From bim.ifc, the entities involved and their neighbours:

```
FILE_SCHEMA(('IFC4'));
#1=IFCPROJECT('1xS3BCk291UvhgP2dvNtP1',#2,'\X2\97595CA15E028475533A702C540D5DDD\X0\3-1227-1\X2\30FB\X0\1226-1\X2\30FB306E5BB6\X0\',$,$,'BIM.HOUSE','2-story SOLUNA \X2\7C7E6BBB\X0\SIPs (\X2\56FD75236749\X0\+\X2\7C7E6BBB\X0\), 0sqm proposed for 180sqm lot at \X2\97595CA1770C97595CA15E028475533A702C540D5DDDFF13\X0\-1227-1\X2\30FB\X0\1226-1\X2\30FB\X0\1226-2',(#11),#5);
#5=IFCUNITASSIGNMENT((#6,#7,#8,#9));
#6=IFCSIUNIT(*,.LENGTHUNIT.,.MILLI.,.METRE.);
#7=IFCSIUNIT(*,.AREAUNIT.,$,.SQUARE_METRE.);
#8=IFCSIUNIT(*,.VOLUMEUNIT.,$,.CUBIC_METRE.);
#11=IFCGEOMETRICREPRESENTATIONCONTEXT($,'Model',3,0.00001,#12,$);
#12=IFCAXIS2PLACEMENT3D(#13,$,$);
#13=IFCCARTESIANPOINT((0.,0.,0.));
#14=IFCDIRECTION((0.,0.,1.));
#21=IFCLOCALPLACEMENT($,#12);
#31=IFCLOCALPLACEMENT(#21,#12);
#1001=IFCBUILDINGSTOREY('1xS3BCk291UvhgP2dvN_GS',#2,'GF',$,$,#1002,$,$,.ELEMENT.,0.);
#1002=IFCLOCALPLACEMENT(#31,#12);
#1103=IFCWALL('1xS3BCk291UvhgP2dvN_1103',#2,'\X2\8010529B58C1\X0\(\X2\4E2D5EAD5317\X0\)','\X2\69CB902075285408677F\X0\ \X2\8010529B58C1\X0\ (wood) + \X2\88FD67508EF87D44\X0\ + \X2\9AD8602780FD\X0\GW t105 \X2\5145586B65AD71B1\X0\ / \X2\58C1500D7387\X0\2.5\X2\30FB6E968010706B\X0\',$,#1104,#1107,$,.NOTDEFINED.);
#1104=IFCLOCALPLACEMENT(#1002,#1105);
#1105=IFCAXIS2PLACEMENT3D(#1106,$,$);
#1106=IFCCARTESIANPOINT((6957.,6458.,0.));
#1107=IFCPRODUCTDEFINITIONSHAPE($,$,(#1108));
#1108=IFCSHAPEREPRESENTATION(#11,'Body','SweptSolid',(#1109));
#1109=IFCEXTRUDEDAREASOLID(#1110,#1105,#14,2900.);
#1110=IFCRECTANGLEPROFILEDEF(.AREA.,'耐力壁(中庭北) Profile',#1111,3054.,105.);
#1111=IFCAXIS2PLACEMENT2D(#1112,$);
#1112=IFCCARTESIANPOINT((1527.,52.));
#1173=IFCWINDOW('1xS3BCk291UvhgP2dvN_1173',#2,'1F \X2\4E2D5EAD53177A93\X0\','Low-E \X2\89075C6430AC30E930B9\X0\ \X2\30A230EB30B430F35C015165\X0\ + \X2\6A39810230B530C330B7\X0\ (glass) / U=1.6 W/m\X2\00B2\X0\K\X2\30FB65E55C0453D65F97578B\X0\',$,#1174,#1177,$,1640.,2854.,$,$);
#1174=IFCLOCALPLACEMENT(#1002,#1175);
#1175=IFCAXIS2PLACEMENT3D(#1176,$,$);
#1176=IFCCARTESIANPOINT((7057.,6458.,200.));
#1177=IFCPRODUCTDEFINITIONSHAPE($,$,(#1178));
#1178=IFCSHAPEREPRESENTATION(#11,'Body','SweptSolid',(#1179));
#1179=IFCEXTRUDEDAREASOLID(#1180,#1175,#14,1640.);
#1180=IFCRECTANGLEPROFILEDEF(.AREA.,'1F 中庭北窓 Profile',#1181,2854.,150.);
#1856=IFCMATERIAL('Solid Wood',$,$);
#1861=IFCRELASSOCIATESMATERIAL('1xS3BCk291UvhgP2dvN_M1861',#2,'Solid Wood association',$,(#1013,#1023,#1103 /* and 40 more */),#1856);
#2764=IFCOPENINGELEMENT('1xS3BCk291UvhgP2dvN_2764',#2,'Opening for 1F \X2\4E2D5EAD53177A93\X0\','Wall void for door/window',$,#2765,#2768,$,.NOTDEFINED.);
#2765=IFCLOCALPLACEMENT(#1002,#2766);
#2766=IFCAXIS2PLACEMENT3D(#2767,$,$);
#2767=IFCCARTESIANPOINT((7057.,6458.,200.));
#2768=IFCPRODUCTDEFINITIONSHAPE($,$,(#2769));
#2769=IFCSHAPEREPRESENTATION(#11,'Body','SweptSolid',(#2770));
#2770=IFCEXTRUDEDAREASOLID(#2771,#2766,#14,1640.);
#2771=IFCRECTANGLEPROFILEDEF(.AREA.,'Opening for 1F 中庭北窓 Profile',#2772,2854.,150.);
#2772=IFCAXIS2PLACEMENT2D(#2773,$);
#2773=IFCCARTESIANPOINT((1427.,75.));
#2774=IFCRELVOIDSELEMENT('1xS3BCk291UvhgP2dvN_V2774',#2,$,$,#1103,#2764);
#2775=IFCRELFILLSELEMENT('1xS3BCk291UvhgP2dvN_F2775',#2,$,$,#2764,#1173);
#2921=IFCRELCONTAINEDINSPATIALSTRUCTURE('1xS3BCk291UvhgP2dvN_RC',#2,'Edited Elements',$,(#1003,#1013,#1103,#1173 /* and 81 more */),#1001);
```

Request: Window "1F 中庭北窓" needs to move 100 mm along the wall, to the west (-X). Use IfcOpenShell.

```python
import ifcopenshell
import ifcopenshell.api.geometry
import ifcopenshell.util.placement

model = ifcopenshell.open("bim.ifc")

window = model.by_guid("1xS3BCk291UvhgP2dvN_1173")
opening = window.FillsVoids[0].RelatingOpeningElement
wall = opening.VoidsElements[0].RelatingBuildingElement

wall_matrix = ifcopenshell.util.placement.get_local_placement(wall.ObjectPlacement)
shift = wall_matrix[:3, 0] * -100.0
before = ifcopenshell.util.placement.get_local_placement(window.ObjectPlacement)[:3, 3].copy()

# The window is not placed relative to its opening, so move both.
for product in (opening, window):
    matrix = ifcopenshell.util.placement.get_local_placement(product.ObjectPlacement)
    matrix[:3, 3] += shift
    ifcopenshell.api.geometry.edit_object_placement(model, product=product, matrix=matrix, is_si=False)

after = ifcopenshell.util.placement.get_local_placement(window.ObjectPlacement)[:3, 3]
print("window moved by", (after - before).round(3) + 0.0)

model.write("bim-out.ifc")
```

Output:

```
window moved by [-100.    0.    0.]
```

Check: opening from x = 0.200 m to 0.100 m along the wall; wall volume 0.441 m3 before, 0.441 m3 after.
